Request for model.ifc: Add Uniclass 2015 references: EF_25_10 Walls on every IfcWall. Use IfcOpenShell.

First a look at what the model holds.

```python
import ifcopenshell

model = ifcopenshell.open("model.ifc")
print(model.schema)
print("classifications:", [c.Name for c in model.by_type("IfcClassification")])
for ifc_class in ("IfcDoor", "IfcRoof", "IfcStair", "IfcWall", "IfcWindow"):
    print(ifc_class, len(model.by_type(ifc_class)))
```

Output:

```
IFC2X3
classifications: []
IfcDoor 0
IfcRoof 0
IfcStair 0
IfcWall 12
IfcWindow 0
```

```python
import ifcopenshell
import ifcopenshell.api.classification

model = ifcopenshell.open("model.ifc")

# IFC2X3 requires Source and Edition and has no link from the project to the system.
system = model.create_entity("IfcClassification", Source="NBS", Edition="2015", Name="Uniclass 2015")

codes = {
    "IfcWall": ("EF_25_10", "Walls"),
}
for ifc_class, (code, name) in codes.items():
    products = model.by_type(ifc_class)
    ifcopenshell.api.classification.add_reference(
        model, products=products, classification=system, identification=code, name=name
    )
    print(code, len(products))

model.write("model_edited.ifc")
```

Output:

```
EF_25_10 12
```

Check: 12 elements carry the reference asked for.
